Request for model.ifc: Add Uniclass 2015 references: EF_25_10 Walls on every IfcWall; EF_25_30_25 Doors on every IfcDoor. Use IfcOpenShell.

First a look at what the model holds.

```python
import ifcopenshell

model = ifcopenshell.open("model.ifc")
print(model.schema)
print("classifications:", [c.Name for c in model.by_type("IfcClassification")])
for ifc_class in ("IfcDoor", "IfcRoof", "IfcStair", "IfcWall", "IfcWindow"):
    print(ifc_class, len(model.by_type(ifc_class)))
```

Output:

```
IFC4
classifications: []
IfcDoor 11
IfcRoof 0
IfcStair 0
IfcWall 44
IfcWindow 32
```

```python
import ifcopenshell
import ifcopenshell.api.classification

model = ifcopenshell.open("model.ifc")

system = ifcopenshell.api.classification.add_classification(model, classification="Uniclass 2015")

codes = {
    "IfcWall": ("EF_25_10", "Walls"),
    "IfcDoor": ("EF_25_30_25", "Doors"),
}
for ifc_class, (code, name) in codes.items():
    products = model.by_type(ifc_class)
    ifcopenshell.api.classification.add_reference(
        model, products=products, classification=system, identification=code, name=name
    )
    print(code, len(products))

model.write("model_updated.ifc")
```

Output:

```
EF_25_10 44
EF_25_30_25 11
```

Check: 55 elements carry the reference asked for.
